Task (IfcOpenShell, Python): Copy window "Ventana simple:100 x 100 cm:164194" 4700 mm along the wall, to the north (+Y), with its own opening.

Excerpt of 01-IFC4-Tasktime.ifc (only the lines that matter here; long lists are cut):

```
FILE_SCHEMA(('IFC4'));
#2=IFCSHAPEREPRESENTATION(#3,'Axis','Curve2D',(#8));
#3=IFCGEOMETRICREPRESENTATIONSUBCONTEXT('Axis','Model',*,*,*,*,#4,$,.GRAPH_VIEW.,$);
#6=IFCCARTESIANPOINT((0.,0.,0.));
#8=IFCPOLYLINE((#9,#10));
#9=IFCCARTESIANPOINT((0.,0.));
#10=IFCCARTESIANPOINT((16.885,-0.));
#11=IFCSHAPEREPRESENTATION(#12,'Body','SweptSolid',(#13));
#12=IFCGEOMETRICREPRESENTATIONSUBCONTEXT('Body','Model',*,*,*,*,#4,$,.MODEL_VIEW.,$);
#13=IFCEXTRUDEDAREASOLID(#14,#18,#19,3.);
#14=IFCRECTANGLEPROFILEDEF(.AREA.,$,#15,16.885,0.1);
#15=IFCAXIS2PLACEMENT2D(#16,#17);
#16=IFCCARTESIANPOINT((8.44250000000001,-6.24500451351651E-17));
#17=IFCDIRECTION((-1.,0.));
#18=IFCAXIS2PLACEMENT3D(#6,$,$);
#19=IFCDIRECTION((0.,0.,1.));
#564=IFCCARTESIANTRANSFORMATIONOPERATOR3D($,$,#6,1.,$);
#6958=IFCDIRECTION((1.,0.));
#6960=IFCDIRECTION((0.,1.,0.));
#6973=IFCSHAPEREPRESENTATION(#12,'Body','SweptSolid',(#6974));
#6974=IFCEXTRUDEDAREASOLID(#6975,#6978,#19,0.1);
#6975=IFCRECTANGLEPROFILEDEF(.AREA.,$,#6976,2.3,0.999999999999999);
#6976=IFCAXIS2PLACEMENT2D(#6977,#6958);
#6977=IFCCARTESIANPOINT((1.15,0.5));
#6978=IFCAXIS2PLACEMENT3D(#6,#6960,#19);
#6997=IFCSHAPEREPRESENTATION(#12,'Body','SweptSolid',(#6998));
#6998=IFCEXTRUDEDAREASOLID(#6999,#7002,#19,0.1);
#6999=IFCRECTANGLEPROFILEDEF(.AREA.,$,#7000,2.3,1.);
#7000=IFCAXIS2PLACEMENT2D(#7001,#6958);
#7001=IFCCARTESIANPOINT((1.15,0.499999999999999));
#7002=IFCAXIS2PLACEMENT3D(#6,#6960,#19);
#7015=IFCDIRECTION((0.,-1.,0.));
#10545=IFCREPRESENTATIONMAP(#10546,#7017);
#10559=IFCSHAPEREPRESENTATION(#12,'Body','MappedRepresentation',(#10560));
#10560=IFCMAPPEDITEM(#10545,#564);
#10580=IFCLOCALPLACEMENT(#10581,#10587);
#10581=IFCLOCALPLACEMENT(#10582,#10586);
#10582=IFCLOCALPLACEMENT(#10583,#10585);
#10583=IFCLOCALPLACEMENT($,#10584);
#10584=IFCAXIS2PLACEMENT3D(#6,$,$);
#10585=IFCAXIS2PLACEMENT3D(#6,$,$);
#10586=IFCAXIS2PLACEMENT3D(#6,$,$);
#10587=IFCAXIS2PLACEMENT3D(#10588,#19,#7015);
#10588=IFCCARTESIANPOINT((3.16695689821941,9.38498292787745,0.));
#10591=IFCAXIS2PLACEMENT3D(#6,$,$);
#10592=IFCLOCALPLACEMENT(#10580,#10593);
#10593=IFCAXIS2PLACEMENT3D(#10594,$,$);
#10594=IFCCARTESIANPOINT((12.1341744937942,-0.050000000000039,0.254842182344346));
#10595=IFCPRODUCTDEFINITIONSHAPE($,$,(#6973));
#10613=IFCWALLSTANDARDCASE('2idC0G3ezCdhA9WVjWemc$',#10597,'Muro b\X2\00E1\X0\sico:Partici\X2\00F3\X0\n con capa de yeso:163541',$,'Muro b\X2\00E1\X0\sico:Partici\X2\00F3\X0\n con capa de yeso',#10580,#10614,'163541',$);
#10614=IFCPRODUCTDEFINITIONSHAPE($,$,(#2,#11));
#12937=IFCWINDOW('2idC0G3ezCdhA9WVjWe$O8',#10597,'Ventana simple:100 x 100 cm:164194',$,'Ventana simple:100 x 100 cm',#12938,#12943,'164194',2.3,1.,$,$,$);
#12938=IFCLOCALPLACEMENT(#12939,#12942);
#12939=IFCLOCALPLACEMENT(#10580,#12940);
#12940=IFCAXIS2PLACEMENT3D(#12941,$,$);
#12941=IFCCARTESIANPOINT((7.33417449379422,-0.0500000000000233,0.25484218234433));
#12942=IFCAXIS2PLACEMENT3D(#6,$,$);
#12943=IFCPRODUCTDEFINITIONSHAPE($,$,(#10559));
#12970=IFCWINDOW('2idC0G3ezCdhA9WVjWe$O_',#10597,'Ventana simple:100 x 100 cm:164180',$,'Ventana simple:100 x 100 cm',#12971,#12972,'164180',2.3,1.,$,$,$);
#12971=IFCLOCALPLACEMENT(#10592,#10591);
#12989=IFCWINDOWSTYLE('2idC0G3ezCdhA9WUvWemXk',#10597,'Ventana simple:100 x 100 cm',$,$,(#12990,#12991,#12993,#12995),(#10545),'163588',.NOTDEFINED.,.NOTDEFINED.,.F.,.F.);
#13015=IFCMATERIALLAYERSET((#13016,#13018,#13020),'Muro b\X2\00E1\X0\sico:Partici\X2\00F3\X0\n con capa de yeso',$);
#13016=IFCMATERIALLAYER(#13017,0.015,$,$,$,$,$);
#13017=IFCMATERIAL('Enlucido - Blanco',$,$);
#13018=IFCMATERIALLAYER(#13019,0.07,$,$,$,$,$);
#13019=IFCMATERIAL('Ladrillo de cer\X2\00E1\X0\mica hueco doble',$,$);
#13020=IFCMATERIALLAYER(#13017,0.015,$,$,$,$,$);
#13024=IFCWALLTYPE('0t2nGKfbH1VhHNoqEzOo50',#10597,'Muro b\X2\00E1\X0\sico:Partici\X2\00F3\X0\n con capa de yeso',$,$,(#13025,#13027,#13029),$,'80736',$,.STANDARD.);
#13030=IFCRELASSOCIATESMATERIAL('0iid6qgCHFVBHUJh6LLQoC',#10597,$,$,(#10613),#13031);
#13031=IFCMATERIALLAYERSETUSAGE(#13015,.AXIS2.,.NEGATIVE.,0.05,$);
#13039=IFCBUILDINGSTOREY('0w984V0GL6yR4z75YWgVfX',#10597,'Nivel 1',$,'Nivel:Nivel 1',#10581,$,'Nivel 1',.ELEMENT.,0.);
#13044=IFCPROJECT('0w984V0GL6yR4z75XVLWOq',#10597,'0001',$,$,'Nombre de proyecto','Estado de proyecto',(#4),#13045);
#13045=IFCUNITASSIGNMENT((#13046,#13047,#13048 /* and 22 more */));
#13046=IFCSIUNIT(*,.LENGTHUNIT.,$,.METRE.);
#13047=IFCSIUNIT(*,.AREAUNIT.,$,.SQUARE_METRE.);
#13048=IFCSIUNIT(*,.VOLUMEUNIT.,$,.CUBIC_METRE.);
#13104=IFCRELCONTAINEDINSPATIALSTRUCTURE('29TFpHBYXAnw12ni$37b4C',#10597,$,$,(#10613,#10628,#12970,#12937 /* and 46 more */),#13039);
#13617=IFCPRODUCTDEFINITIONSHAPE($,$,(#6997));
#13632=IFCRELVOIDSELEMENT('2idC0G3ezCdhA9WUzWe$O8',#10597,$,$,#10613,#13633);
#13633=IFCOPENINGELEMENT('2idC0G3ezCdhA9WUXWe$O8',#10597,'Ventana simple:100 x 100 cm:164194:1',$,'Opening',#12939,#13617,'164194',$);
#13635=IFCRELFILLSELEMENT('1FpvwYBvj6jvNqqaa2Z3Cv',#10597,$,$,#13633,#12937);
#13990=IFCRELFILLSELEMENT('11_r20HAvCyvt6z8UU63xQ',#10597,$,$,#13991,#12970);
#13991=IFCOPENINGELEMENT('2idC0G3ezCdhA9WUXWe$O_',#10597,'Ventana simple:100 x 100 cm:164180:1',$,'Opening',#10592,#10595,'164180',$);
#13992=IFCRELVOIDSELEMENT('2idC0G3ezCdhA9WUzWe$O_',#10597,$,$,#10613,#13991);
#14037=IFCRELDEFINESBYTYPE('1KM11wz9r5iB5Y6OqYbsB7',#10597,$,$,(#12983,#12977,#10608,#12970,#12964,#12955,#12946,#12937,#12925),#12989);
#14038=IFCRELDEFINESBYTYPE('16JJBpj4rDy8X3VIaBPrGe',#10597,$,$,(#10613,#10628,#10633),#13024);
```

```python
import ifcopenshell
import ifcopenshell.api.feature
import ifcopenshell.api.geometry
import ifcopenshell.api.root
import ifcopenshell.geom
import ifcopenshell.util.element
import ifcopenshell.util.placement
import ifcopenshell.util.shape
import ifcopenshell.util.unit

model = ifcopenshell.open("01-IFC4-Tasktime.ifc")
unit_scale = ifcopenshell.util.unit.calculate_unit_scale(model)
settings = ifcopenshell.geom.settings()


def volume(element):
    """Net volume in cubic metres, openings subtracted."""
    shape = ifcopenshell.geom.create_shape(settings, element)
    return ifcopenshell.util.shape.get_volume(shape.geometry)


def reuse_history(source, copy):
    """copy_class also copies each property set's owner history, people and application; keep the originals."""
    for rel in copy.IsDefinedBy:
        if rel.is_a("IfcRelDefinesByProperties") and (history := rel.RelatingPropertyDefinition.OwnerHistory):
            rel.RelatingPropertyDefinition.OwnerHistory = source.OwnerHistory
            ifcopenshell.util.element.remove_deep2(model, history)


window = model.by_guid("2idC0G3ezCdhA9WVjWe$O8")
opening = window.FillsVoids[0].RelatingOpeningElement
wall = opening.VoidsElements[0].RelatingBuildingElement
before = volume(wall)
shift = ifcopenshell.util.placement.get_local_placement(wall.ObjectPlacement)[:3, 0] * -4.7 / unit_scale

# copy_class copies the void relationship, type, container and properties, but no geometry.
new_opening = ifcopenshell.api.root.copy_class(model, product=opening)
new_opening.Representation = ifcopenshell.util.element.copy_deep(
    model, opening.Representation, exclude=["IfcGeometricRepresentationContext", "IfcRepresentationMap"]
)
new_opening.Name = "Ventana simple:100 x 100 cm"
new_opening.Tag = None
new_window = ifcopenshell.api.root.copy_class(model, product=window)
new_window.Representation = ifcopenshell.util.element.copy_deep(
    model, window.Representation, exclude=["IfcGeometricRepresentationContext", "IfcRepresentationMap"]
)
new_window.Name = "Ventana simple:100 x 100 cm"
new_window.Tag = None
reuse_history(window, new_window)
ifcopenshell.api.feature.add_filling(model, opening=new_opening, element=new_window)

for old, new in ((opening, new_opening), (window, new_window)):
    matrix = ifcopenshell.util.placement.get_local_placement(old.ObjectPlacement)
    matrix[:3, 3] += shift
    ifcopenshell.api.geometry.edit_object_placement(model, product=new, matrix=matrix, is_si=False)

after = volume(wall)

print(f"wall volume {before:.3f} -> {after:.3f} m3")

model.write("01-IFC4-Tasktime_edited.ifc")
```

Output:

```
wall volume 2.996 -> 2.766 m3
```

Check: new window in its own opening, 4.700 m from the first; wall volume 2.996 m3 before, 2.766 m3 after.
